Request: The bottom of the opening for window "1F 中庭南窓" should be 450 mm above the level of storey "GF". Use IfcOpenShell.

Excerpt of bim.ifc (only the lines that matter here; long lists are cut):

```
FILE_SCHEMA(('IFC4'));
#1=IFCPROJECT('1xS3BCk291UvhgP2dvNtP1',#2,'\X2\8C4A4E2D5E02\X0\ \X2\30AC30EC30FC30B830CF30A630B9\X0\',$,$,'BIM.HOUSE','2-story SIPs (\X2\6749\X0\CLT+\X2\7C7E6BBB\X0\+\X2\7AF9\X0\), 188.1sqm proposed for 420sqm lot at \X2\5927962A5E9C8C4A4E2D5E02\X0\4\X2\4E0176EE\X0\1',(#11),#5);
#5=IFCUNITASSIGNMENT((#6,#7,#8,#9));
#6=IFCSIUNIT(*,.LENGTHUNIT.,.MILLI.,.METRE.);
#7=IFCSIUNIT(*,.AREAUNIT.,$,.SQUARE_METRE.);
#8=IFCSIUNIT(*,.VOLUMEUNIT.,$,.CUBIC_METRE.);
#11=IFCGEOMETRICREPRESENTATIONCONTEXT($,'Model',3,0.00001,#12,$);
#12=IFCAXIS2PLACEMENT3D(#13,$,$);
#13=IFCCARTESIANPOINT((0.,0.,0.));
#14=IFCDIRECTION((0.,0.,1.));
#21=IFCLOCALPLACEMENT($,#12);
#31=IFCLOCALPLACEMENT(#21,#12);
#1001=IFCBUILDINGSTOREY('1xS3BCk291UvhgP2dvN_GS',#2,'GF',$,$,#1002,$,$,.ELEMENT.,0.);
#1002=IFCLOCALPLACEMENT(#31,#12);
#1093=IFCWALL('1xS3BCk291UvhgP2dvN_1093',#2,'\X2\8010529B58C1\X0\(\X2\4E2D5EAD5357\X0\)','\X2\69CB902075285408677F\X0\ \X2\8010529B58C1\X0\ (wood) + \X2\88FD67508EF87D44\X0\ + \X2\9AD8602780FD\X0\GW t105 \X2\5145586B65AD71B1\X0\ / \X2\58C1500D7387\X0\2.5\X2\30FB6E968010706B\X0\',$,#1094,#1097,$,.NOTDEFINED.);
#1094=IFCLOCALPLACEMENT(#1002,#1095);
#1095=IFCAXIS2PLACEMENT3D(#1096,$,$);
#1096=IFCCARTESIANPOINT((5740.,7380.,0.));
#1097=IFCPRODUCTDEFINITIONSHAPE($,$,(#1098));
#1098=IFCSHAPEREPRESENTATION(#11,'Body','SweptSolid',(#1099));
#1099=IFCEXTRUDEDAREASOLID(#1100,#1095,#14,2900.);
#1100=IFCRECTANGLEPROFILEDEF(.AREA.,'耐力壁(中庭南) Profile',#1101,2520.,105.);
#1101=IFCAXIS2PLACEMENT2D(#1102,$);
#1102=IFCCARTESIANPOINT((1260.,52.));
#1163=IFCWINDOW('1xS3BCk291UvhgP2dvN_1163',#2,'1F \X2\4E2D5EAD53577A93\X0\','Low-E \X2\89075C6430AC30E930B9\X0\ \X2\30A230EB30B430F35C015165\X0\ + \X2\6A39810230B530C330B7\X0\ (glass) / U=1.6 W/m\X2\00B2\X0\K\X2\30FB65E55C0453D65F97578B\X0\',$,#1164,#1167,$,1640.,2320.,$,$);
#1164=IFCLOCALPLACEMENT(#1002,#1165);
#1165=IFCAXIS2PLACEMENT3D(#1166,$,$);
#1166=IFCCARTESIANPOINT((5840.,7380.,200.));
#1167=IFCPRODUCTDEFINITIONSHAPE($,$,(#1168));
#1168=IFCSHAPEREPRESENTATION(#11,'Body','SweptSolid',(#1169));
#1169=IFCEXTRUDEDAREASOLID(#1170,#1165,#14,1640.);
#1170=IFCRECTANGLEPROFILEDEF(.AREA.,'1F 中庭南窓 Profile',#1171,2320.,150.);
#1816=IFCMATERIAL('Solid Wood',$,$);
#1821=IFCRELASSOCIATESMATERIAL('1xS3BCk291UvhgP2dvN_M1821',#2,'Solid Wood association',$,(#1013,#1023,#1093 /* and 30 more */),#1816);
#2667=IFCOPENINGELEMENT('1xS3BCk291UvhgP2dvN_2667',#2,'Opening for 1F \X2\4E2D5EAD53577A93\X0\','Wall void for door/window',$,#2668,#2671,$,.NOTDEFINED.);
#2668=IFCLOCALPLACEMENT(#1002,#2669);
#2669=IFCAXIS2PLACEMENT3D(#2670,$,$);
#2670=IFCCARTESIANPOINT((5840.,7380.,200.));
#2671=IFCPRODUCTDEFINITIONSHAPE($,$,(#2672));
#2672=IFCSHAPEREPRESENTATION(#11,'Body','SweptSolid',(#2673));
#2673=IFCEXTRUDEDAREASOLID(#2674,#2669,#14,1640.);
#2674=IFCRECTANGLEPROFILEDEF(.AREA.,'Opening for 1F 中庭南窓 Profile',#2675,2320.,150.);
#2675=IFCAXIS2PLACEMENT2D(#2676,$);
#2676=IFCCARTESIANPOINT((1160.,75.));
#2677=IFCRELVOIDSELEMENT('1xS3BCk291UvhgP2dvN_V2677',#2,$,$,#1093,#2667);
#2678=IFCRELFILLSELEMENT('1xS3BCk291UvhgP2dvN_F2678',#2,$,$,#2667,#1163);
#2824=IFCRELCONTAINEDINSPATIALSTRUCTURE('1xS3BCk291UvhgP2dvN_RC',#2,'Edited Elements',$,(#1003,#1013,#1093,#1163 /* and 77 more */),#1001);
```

```python
import numpy as np
import ifcopenshell
import ifcopenshell.api.geometry
import ifcopenshell.geom
import ifcopenshell.util.element
import ifcopenshell.util.placement
import ifcopenshell.util.shape
import ifcopenshell.util.unit

model = ifcopenshell.open("bim.ifc")
unit_scale = ifcopenshell.util.unit.calculate_unit_scale(model)

window = model.by_guid("1xS3BCk291UvhgP2dvN_1163")
opening = window.FillsVoids[0].RelatingOpeningElement
storey = ifcopenshell.util.element.get_container(window, ifc_class="IfcBuildingStorey")
level = ifcopenshell.util.placement.get_local_placement(storey.ObjectPlacement)[2, 3]

# The opening's origin need not be at the sill, so measure its lowest point.
shape = ifcopenshell.geom.create_shape(ifcopenshell.geom.settings(), opening)
bottom = ifcopenshell.util.shape.get_shape_bottom_elevation(shape, shape.geometry) / unit_scale
dz = level + 450.0 - bottom

shift = np.array([0.0, 0.0, dz])
# The window is not placed relative to its opening, so move both.
for product in (opening, window):
    matrix = ifcopenshell.util.placement.get_local_placement(product.ObjectPlacement)
    matrix[:3, 3] += shift
    ifcopenshell.api.geometry.edit_object_placement(model, product=product, matrix=matrix, is_si=False)

print(f"moved by {dz * unit_scale:+.3f} m")

model.write("bim_edited.ifc")
```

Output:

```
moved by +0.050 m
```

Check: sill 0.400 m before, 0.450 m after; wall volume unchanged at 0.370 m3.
